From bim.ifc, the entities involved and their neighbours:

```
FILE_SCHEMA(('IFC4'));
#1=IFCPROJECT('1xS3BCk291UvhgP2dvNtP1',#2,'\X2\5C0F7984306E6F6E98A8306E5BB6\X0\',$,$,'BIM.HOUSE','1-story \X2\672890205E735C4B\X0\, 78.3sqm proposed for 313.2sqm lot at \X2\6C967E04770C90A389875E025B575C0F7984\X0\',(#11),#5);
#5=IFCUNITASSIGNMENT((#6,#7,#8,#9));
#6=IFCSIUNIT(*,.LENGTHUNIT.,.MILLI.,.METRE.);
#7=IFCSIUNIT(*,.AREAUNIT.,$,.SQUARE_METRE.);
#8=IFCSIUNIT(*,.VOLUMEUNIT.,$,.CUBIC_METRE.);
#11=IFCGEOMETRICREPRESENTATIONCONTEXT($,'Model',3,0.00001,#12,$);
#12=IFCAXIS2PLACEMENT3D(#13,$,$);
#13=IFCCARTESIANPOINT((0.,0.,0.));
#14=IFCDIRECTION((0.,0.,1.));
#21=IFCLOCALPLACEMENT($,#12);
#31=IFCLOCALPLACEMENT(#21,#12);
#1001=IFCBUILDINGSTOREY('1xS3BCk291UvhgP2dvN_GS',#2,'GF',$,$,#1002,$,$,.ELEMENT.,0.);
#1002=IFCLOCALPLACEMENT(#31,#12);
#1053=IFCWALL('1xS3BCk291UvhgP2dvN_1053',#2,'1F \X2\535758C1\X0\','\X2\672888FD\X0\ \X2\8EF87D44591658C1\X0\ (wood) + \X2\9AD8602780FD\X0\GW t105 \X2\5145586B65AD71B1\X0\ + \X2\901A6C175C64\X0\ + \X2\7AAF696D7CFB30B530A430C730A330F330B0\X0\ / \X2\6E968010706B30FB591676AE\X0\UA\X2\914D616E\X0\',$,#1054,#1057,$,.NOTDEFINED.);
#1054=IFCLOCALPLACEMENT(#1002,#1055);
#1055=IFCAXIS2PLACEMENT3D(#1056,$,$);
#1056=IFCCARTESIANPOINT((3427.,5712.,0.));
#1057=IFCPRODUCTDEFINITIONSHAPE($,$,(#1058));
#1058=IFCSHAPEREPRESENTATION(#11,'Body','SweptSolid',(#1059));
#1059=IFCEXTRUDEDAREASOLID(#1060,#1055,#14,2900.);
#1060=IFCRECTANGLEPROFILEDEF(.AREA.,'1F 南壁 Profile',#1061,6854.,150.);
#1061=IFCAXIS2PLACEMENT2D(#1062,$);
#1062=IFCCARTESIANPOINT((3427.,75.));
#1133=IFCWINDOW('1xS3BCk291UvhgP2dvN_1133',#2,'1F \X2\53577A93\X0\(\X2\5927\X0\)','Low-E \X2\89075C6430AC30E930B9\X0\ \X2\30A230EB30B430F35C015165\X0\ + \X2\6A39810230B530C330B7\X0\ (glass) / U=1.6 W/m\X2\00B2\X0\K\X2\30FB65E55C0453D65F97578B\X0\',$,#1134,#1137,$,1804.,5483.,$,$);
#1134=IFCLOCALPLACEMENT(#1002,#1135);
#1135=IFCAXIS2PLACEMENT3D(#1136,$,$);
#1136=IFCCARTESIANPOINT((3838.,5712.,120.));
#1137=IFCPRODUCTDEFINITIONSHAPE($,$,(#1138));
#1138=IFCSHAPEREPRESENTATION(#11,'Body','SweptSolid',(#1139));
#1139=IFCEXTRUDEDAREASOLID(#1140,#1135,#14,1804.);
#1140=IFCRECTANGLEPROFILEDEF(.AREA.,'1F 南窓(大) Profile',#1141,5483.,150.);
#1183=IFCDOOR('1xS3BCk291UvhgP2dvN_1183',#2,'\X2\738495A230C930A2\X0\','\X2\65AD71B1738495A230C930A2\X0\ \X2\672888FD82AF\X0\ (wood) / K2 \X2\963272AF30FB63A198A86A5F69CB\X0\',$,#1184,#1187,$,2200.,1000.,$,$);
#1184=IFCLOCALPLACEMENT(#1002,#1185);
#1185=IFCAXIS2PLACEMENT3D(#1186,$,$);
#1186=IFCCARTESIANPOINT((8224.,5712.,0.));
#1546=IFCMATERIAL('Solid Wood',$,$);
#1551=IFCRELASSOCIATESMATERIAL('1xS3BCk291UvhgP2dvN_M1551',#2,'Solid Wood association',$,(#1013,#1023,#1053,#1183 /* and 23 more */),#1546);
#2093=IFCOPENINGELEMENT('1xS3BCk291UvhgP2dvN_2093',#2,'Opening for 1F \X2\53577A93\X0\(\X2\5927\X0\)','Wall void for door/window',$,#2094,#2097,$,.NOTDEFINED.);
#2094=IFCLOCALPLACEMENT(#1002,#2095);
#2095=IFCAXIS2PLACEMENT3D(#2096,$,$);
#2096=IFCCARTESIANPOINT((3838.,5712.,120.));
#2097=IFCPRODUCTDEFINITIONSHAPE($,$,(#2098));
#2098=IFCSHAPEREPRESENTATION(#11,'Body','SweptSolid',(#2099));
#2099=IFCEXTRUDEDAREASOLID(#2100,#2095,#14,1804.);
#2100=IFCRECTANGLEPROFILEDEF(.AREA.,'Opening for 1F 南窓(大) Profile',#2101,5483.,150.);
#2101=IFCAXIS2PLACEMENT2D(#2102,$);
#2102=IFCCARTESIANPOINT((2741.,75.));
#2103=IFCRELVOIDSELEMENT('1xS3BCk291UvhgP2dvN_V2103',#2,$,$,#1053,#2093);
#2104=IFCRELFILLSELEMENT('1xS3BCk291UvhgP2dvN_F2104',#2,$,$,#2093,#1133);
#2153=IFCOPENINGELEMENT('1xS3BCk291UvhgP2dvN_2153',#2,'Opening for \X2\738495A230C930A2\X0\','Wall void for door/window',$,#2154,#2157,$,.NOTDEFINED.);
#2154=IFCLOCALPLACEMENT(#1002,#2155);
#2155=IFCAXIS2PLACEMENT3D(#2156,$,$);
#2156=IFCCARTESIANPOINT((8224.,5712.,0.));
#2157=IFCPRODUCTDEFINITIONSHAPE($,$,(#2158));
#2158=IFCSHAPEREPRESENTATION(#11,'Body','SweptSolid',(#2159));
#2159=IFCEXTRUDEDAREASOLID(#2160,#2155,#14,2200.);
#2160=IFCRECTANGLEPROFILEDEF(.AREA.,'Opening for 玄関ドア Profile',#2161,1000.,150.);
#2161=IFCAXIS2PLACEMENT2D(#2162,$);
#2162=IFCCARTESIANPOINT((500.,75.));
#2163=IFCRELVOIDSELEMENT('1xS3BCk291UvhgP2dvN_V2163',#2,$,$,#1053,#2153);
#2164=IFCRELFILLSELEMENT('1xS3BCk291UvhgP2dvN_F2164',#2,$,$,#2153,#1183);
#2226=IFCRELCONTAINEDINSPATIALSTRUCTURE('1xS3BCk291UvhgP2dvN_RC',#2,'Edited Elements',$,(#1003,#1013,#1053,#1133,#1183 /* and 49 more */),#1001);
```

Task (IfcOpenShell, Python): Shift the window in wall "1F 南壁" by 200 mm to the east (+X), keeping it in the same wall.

```python
import ifcopenshell
import ifcopenshell.api.geometry
import ifcopenshell.util.placement

model = ifcopenshell.open("bim.ifc")

window = model.by_guid("1xS3BCk291UvhgP2dvN_1133")
opening = window.FillsVoids[0].RelatingOpeningElement
wall = opening.VoidsElements[0].RelatingBuildingElement

wall_matrix = ifcopenshell.util.placement.get_local_placement(wall.ObjectPlacement)
shift = wall_matrix[:3, 0] * 200.0
before = ifcopenshell.util.placement.get_local_placement(window.ObjectPlacement)[:3, 3].copy()

# The window is not placed relative to its opening, so move both.
for product in (opening, window):
    matrix = ifcopenshell.util.placement.get_local_placement(product.ObjectPlacement)
    matrix[:3, 3] += shift
    ifcopenshell.api.geometry.edit_object_placement(model, product=product, matrix=matrix, is_si=False)

after = ifcopenshell.util.placement.get_local_placement(window.ObjectPlacement)[:3, 3]
print("window moved by", (after - before).round(3) + 0.0)

model.write("bim_v2.ifc")
```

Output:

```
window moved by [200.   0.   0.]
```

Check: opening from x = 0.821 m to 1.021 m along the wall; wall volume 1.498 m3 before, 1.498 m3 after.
